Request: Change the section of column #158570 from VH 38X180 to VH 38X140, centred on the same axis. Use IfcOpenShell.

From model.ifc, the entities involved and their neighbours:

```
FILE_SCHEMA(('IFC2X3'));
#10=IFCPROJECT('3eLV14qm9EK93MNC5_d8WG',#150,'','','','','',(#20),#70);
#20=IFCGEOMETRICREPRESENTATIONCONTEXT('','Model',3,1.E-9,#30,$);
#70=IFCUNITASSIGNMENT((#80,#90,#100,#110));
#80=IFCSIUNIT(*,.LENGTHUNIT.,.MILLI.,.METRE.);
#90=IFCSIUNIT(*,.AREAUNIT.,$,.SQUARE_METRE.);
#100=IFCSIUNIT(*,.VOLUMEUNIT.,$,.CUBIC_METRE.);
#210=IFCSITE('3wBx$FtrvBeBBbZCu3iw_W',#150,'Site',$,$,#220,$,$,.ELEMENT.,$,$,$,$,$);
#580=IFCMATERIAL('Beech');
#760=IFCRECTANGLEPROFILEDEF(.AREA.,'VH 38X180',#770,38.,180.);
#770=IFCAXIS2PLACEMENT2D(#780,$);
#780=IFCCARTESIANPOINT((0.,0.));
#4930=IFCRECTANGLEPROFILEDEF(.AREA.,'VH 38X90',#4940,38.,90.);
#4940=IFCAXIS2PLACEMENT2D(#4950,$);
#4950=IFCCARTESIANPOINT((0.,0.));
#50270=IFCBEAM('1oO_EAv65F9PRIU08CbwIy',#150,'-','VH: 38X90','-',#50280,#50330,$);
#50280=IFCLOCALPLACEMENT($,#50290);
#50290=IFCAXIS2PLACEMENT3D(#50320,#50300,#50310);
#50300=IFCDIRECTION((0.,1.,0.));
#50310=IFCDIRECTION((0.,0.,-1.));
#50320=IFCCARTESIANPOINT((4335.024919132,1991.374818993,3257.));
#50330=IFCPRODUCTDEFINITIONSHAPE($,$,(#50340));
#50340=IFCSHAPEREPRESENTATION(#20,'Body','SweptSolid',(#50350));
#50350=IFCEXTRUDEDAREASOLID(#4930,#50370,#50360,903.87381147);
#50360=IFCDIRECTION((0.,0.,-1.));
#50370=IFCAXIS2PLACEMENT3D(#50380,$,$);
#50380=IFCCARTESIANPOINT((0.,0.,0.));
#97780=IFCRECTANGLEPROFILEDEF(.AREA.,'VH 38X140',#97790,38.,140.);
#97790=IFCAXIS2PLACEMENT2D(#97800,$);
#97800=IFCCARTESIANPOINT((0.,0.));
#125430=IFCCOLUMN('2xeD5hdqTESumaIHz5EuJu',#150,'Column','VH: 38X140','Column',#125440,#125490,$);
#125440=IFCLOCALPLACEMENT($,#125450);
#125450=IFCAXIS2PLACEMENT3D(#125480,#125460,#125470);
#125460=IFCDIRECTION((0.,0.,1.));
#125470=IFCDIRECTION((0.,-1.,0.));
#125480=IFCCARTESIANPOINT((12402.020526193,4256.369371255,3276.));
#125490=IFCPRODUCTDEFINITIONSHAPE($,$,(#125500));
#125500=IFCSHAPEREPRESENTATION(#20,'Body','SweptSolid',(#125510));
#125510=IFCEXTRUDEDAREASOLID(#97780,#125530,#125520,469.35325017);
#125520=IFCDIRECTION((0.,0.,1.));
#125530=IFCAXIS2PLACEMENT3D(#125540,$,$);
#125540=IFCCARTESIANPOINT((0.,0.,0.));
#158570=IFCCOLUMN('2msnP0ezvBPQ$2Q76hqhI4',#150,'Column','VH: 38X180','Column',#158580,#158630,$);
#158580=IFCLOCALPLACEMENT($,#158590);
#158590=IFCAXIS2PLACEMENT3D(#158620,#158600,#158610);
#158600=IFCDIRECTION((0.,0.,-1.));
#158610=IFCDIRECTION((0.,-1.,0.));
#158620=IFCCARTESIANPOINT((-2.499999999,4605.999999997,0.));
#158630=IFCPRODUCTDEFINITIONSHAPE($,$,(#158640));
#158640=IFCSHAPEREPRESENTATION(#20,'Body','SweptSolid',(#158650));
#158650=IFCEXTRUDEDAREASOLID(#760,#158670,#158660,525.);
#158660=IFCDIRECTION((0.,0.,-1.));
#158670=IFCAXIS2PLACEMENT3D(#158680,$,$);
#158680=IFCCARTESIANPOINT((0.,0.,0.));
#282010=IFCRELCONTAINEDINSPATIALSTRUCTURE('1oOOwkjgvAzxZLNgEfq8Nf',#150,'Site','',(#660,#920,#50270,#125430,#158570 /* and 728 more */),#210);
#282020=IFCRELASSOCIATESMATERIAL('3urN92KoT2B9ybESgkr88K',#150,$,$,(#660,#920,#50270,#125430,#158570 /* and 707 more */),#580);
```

```python
import ifcopenshell
import ifcopenshell.util.element

model = ifcopenshell.open("model.ifc")

member = model.by_guid("2msnP0ezvBPQ$2Q76hqhI4")
source = next(p for p in model.by_type("IfcRectangleProfileDef") if p.ProfileName == "VH 38X140")

body = next(r for r in member.Representation.Representations if r.RepresentationIdentifier == "Body")
solid = body.Items[0]
old_profile = solid.SweptArea

# Copy the section's sizes but keep this member's own profile position.
profile = ifcopenshell.util.element.copy(model, source)
profile.Position = old_profile.Position
solid.SweptArea = profile
if not model.get_total_inverses(old_profile):
    ifcopenshell.util.element.remove_deep2(model, old_profile)

print(solid.SweptArea)

model.write("model_updated.ifc")
```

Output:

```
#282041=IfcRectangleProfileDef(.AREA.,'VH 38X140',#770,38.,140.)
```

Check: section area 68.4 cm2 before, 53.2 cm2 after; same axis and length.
